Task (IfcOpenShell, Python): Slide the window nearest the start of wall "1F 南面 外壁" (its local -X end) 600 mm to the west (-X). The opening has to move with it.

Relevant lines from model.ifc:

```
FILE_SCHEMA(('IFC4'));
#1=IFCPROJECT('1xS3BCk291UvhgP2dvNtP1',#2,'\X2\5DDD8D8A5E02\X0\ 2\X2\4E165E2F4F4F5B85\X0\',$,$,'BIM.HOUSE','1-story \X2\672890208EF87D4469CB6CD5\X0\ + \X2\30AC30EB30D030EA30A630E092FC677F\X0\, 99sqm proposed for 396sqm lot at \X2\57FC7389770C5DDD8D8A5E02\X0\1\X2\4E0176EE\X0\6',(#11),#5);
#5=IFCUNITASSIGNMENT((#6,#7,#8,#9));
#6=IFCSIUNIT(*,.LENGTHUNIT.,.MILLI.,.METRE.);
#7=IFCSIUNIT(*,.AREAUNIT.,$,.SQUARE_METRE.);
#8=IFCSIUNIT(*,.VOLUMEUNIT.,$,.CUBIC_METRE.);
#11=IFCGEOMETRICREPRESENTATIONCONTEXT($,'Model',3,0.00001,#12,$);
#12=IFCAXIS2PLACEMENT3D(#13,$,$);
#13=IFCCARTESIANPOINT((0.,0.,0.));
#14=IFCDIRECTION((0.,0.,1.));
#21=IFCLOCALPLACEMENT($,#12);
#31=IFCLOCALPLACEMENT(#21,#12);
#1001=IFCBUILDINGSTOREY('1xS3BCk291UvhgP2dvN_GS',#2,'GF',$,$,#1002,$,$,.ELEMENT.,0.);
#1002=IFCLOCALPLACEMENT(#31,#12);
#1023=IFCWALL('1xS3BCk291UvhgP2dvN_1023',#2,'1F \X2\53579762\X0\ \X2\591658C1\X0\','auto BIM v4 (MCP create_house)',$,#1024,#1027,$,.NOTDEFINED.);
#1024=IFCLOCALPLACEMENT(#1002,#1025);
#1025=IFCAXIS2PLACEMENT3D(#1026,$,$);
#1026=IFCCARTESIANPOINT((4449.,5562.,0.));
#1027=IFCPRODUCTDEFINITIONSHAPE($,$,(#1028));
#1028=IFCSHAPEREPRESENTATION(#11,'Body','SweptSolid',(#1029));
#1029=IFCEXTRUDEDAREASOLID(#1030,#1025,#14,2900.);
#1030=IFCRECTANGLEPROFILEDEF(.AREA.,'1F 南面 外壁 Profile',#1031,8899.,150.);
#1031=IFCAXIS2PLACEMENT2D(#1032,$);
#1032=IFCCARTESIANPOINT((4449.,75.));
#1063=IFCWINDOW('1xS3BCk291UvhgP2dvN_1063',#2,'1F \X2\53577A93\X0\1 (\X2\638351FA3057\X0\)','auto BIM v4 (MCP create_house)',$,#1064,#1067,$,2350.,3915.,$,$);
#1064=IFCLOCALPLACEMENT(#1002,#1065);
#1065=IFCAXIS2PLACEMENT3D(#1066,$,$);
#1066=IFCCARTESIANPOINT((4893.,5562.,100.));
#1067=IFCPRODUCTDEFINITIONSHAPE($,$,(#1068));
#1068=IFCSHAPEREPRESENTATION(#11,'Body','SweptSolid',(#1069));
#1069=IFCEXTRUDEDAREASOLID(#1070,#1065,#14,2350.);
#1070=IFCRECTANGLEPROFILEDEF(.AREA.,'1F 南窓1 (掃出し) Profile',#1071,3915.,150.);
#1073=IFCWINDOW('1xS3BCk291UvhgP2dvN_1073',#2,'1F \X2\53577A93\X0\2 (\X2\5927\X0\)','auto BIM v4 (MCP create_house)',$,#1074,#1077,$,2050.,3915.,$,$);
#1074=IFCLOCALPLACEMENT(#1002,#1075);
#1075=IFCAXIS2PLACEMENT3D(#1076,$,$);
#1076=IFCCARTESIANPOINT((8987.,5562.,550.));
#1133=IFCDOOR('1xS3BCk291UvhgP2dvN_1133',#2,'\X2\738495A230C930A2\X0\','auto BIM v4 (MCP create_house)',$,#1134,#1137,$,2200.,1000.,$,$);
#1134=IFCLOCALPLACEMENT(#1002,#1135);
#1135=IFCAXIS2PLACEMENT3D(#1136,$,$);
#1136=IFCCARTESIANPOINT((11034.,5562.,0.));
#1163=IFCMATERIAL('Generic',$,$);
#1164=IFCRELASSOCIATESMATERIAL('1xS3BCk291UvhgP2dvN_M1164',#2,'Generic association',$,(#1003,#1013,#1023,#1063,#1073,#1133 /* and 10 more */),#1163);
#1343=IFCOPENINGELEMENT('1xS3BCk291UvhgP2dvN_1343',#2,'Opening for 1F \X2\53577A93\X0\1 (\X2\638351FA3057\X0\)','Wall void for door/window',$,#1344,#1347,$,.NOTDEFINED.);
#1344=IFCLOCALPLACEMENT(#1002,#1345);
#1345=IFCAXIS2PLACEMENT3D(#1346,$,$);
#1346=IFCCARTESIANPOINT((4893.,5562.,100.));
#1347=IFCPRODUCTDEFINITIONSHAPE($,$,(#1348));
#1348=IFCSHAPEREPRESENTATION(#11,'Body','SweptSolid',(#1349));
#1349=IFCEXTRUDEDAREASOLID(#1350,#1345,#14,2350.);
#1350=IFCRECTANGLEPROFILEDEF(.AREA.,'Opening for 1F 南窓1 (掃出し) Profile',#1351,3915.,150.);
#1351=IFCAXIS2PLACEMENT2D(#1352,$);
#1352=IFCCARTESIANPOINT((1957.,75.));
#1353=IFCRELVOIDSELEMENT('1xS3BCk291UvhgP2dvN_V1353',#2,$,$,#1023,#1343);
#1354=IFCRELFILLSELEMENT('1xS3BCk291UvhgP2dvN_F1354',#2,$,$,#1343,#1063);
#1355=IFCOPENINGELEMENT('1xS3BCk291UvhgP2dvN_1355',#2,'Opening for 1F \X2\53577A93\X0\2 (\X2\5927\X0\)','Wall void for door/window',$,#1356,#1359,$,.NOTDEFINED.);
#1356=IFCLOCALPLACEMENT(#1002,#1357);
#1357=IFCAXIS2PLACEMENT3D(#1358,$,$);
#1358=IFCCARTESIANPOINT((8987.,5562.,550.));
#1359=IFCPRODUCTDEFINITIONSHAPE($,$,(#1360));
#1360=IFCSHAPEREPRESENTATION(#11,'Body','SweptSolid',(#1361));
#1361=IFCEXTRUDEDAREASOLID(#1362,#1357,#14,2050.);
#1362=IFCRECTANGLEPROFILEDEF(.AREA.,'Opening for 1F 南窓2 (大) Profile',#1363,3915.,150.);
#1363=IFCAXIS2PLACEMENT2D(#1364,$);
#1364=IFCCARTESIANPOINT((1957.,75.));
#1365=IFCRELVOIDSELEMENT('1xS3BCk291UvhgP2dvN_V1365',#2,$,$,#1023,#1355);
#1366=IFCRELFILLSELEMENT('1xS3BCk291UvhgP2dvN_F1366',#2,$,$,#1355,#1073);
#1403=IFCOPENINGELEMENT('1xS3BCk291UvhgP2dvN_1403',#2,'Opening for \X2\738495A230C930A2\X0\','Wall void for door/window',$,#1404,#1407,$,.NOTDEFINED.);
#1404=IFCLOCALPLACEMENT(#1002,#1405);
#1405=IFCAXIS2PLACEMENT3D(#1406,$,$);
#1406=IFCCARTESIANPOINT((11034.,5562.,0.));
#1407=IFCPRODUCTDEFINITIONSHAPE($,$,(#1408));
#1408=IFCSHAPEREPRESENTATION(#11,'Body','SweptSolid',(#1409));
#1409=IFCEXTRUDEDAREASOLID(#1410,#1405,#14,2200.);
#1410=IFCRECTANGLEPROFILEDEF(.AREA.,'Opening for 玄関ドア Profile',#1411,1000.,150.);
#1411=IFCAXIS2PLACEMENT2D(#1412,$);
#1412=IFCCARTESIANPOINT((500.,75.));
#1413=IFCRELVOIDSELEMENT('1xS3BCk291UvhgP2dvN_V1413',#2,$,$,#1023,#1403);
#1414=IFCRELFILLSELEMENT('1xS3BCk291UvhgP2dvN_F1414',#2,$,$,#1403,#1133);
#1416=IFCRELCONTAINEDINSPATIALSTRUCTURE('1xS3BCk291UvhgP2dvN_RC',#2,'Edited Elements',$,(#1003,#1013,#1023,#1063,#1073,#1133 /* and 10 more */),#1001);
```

```python
import ifcopenshell
import ifcopenshell.api.geometry
import ifcopenshell.util.placement

model = ifcopenshell.open("model.ifc")

window = model.by_guid("1xS3BCk291UvhgP2dvN_1063")
opening = window.FillsVoids[0].RelatingOpeningElement
wall = opening.VoidsElements[0].RelatingBuildingElement

wall_matrix = ifcopenshell.util.placement.get_local_placement(wall.ObjectPlacement)
shift = wall_matrix[:3, 0] * -600.0
before = ifcopenshell.util.placement.get_local_placement(window.ObjectPlacement)[:3, 3].copy()

# The window is not placed relative to its opening, so move both.
for product in (opening, window):
    matrix = ifcopenshell.util.placement.get_local_placement(product.ObjectPlacement)
    matrix[:3, 3] += shift
    ifcopenshell.api.geometry.edit_object_placement(model, product=product, matrix=matrix, is_si=False)

after = ifcopenshell.util.placement.get_local_placement(window.ObjectPlacement)[:3, 3]
print("window moved by", (after - before).round(3) + 0.0)

model.write("model_updated.ifc")
```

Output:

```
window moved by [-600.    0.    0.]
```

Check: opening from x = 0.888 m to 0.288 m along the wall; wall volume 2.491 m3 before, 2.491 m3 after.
